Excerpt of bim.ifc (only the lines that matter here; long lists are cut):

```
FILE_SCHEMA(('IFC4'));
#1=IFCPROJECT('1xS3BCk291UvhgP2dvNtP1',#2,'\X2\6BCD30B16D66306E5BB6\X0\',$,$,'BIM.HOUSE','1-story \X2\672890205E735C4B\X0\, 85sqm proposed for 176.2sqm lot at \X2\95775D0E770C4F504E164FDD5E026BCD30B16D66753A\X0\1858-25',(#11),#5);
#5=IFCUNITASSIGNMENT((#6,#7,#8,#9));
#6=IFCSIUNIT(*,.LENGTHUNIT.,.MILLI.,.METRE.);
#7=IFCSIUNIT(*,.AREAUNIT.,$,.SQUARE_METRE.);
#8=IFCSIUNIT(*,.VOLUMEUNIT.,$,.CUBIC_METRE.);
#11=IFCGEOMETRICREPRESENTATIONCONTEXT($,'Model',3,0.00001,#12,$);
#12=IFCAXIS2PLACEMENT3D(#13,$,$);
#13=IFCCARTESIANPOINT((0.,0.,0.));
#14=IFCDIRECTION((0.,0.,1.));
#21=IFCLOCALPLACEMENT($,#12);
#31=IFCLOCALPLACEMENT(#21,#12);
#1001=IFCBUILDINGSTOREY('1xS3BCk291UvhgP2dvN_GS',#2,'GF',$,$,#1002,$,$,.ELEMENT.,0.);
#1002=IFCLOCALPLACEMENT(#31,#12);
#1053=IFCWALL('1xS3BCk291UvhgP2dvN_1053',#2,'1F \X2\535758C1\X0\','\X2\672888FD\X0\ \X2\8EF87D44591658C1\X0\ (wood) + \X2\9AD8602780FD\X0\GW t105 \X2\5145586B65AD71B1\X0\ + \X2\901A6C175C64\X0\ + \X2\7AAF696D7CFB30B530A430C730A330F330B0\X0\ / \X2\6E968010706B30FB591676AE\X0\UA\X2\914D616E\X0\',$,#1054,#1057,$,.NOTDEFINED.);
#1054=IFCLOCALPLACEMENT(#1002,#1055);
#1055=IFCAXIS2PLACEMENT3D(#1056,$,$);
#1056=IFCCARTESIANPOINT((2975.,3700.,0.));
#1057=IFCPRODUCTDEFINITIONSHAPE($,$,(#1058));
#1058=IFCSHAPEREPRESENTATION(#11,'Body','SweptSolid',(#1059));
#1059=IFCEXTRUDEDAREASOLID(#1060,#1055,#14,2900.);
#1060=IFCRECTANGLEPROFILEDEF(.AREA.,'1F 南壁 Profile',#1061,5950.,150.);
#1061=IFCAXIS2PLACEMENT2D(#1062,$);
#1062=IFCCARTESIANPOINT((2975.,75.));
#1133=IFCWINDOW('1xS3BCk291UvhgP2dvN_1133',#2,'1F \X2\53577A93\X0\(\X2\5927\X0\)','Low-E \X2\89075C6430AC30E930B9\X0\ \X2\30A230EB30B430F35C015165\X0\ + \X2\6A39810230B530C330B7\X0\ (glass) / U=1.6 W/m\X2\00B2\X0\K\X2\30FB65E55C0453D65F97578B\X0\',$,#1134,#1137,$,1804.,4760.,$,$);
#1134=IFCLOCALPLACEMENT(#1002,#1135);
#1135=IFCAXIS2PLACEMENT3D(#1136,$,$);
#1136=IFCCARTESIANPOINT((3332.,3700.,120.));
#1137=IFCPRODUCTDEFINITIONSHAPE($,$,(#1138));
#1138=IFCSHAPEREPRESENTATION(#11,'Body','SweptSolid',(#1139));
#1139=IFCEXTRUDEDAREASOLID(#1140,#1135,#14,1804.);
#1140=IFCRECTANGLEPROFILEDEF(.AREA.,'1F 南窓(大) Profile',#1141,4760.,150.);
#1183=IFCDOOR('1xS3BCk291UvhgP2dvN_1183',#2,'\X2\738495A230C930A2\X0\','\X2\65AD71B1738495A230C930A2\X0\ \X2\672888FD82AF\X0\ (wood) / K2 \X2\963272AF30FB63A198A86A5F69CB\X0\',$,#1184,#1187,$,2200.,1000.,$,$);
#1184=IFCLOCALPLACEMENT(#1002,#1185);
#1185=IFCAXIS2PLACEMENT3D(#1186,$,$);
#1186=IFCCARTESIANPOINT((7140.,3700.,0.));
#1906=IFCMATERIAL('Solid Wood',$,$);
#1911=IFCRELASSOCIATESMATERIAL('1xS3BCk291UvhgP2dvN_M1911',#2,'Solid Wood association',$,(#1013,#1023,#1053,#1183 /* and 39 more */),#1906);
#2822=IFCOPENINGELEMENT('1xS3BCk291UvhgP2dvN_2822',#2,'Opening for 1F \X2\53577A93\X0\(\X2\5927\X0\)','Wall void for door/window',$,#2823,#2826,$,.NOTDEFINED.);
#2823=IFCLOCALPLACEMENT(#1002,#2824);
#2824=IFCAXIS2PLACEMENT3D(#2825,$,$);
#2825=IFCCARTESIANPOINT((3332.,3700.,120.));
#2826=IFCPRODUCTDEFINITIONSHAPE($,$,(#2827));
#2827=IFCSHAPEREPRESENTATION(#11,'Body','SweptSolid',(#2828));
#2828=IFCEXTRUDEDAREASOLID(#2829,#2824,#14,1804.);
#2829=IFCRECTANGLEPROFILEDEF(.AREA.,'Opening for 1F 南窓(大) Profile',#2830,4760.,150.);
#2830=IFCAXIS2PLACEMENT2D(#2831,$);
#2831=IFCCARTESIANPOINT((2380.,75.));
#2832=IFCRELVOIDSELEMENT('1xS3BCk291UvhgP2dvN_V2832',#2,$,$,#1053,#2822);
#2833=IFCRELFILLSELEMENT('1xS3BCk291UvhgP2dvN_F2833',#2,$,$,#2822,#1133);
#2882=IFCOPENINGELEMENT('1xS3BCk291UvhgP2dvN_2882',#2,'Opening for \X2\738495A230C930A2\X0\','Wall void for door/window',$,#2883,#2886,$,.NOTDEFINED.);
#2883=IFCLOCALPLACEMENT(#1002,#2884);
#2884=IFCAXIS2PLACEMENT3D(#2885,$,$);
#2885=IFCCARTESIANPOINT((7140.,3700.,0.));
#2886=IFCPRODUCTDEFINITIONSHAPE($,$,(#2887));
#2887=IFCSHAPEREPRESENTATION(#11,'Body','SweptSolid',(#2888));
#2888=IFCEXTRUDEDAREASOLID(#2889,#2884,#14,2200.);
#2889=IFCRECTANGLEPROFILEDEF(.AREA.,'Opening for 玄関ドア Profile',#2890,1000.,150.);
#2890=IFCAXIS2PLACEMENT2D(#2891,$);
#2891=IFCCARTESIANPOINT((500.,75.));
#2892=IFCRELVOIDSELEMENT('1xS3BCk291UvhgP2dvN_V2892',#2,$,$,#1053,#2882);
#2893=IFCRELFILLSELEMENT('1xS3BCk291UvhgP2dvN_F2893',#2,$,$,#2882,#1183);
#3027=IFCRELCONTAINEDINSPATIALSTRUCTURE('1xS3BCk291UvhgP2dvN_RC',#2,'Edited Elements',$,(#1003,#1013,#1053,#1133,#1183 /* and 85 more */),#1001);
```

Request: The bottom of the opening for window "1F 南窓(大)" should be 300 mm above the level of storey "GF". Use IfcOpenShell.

```python
import numpy as np
import ifcopenshell
import ifcopenshell.api.geometry
import ifcopenshell.geom
import ifcopenshell.util.element
import ifcopenshell.util.placement
import ifcopenshell.util.shape
import ifcopenshell.util.unit

model = ifcopenshell.open("bim.ifc")
unit_scale = ifcopenshell.util.unit.calculate_unit_scale(model)

window = model.by_guid("1xS3BCk291UvhgP2dvN_1133")
opening = window.FillsVoids[0].RelatingOpeningElement
storey = ifcopenshell.util.element.get_container(window, ifc_class="IfcBuildingStorey")
level = ifcopenshell.util.placement.get_local_placement(storey.ObjectPlacement)[2, 3]

# The opening's origin need not be at the sill, so measure its lowest point.
shape = ifcopenshell.geom.create_shape(ifcopenshell.geom.settings(), opening)
bottom = ifcopenshell.util.shape.get_shape_bottom_elevation(shape, shape.geometry) / unit_scale
dz = level + 0.3 / unit_scale - bottom

shift = np.array([0.0, 0.0, dz])
# The window is not placed relative to its opening, so move both.
for product in (opening, window):
    matrix = ifcopenshell.util.placement.get_local_placement(product.ObjectPlacement)
    matrix[:3, 3] += shift
    ifcopenshell.api.geometry.edit_object_placement(model, product=product, matrix=matrix, is_si=False)

print(f"moved by {dz * unit_scale:+.3f} m")

model.write("bim_rev.ifc")
```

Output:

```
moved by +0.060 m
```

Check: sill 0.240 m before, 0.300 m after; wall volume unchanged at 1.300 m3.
